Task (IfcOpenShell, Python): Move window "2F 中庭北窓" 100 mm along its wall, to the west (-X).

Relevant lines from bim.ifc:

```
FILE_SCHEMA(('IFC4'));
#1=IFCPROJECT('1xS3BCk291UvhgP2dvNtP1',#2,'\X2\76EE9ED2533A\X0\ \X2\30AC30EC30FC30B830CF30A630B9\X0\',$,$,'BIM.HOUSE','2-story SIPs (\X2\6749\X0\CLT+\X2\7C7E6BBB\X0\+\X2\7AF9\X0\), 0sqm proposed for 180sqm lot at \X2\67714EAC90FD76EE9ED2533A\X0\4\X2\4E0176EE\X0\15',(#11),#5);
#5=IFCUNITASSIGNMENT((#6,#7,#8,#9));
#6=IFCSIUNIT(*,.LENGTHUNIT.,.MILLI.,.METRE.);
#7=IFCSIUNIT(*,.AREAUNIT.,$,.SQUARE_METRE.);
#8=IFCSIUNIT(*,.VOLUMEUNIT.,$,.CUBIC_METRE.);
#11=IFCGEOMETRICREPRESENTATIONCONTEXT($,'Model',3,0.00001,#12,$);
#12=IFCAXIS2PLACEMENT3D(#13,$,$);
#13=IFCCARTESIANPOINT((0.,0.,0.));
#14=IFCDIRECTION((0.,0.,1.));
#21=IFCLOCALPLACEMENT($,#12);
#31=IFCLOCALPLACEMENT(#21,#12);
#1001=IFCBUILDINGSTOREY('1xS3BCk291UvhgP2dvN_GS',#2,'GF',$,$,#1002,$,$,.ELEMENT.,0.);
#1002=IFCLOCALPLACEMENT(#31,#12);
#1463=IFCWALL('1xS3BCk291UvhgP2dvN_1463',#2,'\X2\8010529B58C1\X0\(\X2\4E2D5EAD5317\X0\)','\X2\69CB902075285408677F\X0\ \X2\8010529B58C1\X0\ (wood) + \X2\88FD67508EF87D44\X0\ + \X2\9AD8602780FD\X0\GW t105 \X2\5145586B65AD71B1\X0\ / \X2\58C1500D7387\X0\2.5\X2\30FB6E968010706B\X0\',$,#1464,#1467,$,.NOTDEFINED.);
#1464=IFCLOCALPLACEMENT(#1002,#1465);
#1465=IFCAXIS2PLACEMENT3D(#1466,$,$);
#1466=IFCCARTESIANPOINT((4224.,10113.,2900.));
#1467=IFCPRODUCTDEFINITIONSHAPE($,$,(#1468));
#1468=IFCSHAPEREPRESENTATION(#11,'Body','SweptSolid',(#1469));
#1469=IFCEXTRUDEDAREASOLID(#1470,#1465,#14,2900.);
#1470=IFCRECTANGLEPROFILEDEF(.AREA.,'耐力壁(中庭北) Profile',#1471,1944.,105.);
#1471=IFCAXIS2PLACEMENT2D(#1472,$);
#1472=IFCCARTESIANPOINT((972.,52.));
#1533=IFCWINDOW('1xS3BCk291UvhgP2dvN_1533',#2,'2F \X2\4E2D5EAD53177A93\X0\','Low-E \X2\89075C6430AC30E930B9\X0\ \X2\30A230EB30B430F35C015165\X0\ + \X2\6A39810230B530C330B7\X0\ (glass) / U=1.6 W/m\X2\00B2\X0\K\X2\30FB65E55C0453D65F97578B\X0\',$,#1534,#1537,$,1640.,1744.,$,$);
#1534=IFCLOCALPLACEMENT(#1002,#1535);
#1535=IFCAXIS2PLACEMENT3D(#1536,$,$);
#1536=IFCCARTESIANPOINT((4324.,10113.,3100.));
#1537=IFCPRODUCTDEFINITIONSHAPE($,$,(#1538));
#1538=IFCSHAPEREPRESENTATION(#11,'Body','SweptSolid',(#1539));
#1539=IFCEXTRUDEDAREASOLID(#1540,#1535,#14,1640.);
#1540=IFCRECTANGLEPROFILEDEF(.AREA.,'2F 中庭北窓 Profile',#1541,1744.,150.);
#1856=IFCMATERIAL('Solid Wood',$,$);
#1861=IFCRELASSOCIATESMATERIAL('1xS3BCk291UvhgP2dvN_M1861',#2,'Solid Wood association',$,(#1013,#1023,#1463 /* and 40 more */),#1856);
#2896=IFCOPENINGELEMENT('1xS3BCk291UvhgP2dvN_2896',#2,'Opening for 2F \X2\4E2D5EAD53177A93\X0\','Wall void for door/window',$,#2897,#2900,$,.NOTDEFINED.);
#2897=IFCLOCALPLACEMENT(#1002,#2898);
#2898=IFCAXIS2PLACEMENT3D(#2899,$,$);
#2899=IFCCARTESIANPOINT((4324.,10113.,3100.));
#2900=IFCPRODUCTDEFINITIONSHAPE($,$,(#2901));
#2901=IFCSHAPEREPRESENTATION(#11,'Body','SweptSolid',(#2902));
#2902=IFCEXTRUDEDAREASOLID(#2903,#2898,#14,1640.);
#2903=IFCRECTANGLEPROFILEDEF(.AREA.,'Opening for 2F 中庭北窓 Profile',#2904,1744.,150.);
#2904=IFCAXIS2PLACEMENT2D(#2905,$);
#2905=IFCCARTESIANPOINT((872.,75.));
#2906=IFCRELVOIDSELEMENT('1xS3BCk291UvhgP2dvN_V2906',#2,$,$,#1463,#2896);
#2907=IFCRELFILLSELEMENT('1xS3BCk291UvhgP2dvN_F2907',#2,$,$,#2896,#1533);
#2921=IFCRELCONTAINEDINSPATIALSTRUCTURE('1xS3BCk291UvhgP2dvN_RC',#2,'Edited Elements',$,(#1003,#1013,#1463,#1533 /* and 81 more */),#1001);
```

```python
import ifcopenshell
import ifcopenshell.api.geometry
import ifcopenshell.util.placement
import ifcopenshell.util.unit

model = ifcopenshell.open("bim.ifc")
unit_scale = ifcopenshell.util.unit.calculate_unit_scale(model)

window = model.by_guid("1xS3BCk291UvhgP2dvN_1533")
opening = window.FillsVoids[0].RelatingOpeningElement
wall = opening.VoidsElements[0].RelatingBuildingElement

wall_matrix = ifcopenshell.util.placement.get_local_placement(wall.ObjectPlacement)
shift = wall_matrix[:3, 0] * -0.1 / unit_scale
before = ifcopenshell.util.placement.get_local_placement(window.ObjectPlacement)[:3, 3].copy()

# The window is not placed relative to its opening, so move both.
for product in (opening, window):
    matrix = ifcopenshell.util.placement.get_local_placement(product.ObjectPlacement)
    matrix[:3, 3] += shift
    ifcopenshell.api.geometry.edit_object_placement(model, product=product, matrix=matrix, is_si=False)

after = ifcopenshell.util.placement.get_local_placement(window.ObjectPlacement)[:3, 3]
print("window moved by", (after - before).round(3) + 0.0)

model.write("bim-out.ifc")
```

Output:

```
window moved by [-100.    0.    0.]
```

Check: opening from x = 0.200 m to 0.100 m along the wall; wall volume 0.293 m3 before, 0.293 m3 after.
